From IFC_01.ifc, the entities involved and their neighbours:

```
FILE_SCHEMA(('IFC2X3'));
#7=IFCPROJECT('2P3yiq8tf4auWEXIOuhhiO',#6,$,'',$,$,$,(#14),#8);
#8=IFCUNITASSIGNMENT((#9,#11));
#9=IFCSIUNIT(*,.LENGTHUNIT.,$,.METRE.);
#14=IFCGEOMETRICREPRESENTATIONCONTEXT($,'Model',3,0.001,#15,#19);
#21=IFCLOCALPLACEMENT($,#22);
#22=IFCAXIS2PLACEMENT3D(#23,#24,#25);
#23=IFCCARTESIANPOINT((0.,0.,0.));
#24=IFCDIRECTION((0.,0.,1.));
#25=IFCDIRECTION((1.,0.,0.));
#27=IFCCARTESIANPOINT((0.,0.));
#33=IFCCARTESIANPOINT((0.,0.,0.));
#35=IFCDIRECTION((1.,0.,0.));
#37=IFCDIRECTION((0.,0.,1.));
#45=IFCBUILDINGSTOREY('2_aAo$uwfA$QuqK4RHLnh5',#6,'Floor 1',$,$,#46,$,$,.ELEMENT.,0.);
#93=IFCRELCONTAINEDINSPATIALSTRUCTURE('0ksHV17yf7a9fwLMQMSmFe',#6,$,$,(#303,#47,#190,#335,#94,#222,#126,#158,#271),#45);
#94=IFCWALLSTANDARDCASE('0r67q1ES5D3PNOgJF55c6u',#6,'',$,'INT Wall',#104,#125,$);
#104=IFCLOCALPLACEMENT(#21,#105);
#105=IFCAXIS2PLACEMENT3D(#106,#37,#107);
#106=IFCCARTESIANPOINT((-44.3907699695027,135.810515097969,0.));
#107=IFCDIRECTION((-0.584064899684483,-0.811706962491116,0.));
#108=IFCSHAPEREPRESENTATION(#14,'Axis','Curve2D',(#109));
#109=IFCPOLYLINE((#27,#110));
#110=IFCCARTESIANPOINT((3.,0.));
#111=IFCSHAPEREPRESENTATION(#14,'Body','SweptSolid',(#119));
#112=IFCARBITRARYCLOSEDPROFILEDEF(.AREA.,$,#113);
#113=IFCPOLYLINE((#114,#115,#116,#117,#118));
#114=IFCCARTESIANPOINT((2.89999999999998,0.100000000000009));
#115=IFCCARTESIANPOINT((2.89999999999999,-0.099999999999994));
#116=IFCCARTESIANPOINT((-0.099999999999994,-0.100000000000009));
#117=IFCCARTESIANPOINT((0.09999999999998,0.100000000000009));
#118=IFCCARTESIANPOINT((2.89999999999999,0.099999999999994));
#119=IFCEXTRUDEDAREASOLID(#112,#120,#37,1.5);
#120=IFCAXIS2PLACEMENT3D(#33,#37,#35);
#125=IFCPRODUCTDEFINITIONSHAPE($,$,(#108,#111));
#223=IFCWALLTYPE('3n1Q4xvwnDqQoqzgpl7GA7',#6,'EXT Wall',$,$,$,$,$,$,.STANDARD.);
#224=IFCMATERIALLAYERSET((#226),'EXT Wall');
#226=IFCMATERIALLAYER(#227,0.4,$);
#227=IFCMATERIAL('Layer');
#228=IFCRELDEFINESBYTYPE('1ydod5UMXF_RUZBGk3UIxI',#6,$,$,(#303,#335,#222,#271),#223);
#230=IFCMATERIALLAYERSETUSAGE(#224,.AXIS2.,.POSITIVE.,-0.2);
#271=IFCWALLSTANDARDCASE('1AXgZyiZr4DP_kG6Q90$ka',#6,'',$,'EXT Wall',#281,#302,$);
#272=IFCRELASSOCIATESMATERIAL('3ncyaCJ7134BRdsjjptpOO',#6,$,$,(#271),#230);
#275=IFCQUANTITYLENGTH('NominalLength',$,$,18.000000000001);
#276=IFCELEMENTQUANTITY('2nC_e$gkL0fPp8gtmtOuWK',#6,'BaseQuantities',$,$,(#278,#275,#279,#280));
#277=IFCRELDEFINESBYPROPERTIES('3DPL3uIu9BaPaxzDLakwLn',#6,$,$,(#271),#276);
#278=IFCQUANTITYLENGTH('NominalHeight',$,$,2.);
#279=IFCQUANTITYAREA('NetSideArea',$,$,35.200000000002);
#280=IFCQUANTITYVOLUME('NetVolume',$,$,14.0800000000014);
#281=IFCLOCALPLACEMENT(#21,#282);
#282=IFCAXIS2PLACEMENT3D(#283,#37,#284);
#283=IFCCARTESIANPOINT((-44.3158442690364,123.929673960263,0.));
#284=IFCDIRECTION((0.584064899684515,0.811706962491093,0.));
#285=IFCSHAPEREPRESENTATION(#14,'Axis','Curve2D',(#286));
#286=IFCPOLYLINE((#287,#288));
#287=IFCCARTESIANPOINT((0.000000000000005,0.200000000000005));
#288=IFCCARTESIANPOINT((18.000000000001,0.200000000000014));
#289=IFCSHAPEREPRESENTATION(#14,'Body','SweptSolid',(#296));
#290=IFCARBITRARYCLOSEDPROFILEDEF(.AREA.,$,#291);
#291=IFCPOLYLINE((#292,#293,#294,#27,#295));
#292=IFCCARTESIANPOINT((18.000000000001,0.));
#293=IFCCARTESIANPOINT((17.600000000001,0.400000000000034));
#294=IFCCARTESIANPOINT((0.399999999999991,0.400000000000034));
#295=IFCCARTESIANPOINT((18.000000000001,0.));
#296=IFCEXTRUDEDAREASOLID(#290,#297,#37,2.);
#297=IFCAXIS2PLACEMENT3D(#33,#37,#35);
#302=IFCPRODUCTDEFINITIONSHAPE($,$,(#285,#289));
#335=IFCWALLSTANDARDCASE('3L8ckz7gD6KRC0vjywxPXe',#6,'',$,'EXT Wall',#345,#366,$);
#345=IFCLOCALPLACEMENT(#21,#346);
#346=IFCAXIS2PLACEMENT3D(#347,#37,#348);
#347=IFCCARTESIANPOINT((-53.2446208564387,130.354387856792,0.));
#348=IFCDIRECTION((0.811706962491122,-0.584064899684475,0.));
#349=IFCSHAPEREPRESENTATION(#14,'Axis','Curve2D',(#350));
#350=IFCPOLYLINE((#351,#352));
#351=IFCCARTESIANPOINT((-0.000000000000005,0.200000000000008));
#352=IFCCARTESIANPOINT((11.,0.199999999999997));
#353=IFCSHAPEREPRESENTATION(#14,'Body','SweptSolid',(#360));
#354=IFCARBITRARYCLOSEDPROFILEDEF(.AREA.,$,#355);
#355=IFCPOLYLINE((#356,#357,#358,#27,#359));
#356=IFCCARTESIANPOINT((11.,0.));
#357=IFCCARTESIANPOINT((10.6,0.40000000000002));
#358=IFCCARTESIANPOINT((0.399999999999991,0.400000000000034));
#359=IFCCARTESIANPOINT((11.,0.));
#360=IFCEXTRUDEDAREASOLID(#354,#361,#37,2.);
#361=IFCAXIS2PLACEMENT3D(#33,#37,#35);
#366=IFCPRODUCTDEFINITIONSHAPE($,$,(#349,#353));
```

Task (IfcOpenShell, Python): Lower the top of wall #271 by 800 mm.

```python
import ifcopenshell
import ifcopenshell.api.pset
import ifcopenshell.geom
import ifcopenshell.util.element
import ifcopenshell.util.shape
import ifcopenshell.util.unit

model = ifcopenshell.open("IFC_01.ifc")
unit_scale = ifcopenshell.util.unit.calculate_unit_scale(model)
area_scale = ifcopenshell.util.unit.calculate_unit_scale(model, "AREAUNIT")
volume_scale = ifcopenshell.util.unit.calculate_unit_scale(model, "VOLUMEUNIT")
settings = ifcopenshell.geom.settings()


def volume(element):
    """Net volume in cubic metres, openings subtracted."""
    shape = ifcopenshell.geom.create_shape(settings, element)
    return ifcopenshell.util.shape.get_volume(shape.geometry)


wall = model.by_guid("1AXgZyiZr4DP_kG6Q90$ka")
before = volume(wall)

body = next(r for r in wall.Representation.Representations if r.RepresentationIdentifier == "Body")
solid = body.Items[0]
old_height = solid.Depth
solid.Depth -= 0.8 / unit_scale
after = volume(wall)
thickness = 0.4  # wall thickness in metres

# Update the stored height, areas and volumes.
qto = model.by_id(ifcopenshell.util.element.get_pset(wall, "BaseQuantities", should_inherit=False)["id"])
ifcopenshell.api.pset.edit_qto(model, qto=qto, properties={
    "NominalHeight": solid.Depth,
    "NetSideArea": after / thickness / area_scale,
    "NetVolume": after / volume_scale,
})

print(f"height {old_height:g} -> {solid.Depth:g}, volume {before:.3f} -> {after:.3f} m3")

model.write("IFC_01_edited.ifc")
```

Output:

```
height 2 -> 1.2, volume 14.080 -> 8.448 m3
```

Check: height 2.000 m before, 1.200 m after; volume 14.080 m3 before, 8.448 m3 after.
